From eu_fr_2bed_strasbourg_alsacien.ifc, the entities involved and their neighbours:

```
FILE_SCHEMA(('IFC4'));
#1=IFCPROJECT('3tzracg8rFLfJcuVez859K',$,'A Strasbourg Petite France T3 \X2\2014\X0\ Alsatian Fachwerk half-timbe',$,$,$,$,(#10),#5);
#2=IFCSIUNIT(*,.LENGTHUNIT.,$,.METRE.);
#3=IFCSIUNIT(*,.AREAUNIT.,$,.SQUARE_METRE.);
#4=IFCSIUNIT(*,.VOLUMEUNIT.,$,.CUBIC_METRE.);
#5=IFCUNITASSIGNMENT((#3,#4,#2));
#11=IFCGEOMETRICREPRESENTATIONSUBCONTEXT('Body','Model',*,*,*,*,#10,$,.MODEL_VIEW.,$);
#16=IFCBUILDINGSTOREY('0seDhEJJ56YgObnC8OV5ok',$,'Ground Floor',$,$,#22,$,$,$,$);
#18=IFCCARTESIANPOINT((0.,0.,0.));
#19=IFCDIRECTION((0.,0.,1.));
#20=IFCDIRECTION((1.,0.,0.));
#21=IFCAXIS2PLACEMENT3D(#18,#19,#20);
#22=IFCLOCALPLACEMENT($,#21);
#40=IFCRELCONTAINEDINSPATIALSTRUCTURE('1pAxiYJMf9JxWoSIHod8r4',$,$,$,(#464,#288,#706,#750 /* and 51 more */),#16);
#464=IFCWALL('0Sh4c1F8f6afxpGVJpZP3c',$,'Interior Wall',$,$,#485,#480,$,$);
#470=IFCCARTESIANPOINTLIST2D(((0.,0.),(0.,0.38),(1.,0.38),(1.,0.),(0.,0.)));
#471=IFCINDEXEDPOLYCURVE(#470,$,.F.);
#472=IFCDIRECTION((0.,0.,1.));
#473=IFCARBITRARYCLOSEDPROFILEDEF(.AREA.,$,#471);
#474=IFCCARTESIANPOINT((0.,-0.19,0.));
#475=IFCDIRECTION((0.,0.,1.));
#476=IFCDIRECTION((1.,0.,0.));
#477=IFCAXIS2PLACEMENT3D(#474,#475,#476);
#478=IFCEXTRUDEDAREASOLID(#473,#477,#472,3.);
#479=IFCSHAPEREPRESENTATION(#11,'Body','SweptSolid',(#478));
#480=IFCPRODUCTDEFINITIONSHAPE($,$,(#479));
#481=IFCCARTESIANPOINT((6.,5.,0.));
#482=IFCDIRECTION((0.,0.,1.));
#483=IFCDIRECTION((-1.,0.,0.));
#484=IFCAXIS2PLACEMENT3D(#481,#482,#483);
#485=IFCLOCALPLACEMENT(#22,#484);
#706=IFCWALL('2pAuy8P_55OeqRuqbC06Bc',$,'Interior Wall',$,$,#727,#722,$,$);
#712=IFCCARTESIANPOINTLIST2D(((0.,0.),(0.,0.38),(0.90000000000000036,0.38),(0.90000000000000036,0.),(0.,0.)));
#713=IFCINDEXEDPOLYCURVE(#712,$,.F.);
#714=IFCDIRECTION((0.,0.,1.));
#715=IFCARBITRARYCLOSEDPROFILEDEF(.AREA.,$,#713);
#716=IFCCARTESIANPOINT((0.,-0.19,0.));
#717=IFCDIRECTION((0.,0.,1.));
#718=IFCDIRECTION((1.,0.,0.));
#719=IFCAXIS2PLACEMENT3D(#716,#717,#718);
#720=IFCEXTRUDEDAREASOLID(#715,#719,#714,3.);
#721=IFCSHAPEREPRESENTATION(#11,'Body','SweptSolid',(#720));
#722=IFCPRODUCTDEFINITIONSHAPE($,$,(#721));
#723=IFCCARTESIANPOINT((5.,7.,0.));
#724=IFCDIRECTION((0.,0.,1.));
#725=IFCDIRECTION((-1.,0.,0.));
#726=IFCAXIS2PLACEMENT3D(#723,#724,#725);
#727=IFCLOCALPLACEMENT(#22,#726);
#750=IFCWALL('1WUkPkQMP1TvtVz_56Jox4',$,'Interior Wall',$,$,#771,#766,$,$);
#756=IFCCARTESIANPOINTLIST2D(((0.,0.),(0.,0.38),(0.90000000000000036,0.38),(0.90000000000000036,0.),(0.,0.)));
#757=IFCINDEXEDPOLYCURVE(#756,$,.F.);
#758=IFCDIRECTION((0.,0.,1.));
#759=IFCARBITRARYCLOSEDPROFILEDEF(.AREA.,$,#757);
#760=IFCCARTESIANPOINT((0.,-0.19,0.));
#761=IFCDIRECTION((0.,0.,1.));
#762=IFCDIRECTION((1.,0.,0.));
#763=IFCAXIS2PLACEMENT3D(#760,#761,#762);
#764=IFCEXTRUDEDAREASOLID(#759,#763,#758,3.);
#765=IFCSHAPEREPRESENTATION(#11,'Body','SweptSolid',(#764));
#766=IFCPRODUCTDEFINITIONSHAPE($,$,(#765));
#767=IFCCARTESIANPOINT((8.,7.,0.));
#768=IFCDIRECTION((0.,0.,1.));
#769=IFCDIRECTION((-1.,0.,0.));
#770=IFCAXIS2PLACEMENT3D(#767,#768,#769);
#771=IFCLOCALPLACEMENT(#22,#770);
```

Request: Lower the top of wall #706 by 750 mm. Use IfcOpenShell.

```python
import ifcopenshell
import ifcopenshell.geom
import ifcopenshell.util.representation
import ifcopenshell.util.shape

model = ifcopenshell.open("eu_fr_2bed_strasbourg_alsacien.ifc")
settings = ifcopenshell.geom.settings()


def volume(element):
    """Net volume in cubic metres, openings subtracted."""
    shape = ifcopenshell.geom.create_shape(settings, element)
    return ifcopenshell.util.shape.get_volume(shape.geometry)


wall = model.by_guid("2pAuy8P_55OeqRuqbC06Bc")
before = volume(wall)

body = ifcopenshell.util.representation.get_representation(wall, "Model", "Body")
solid = body.Items[0]
old_height = solid.Depth
solid.Depth -= 0.75
after = volume(wall)

print(f"height {old_height:g} -> {solid.Depth:g}, volume {before:.3f} -> {after:.3f} m3")

model.write("eu_fr_2bed_strasbourg_alsacien_rev.ifc")
```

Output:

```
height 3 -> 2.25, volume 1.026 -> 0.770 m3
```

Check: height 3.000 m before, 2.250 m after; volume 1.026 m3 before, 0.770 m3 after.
